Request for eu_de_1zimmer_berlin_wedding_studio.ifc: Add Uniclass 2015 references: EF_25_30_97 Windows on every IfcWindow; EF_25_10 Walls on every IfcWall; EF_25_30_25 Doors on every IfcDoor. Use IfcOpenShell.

First a look at what the model holds.

```python
import ifcopenshell

model = ifcopenshell.open("eu_de_1zimmer_berlin_wedding_studio.ifc")
print(model.schema)
print("classifications:", [c.Name for c in model.by_type("IfcClassification")])
for ifc_class in ("IfcDoor", "IfcRoof", "IfcStair", "IfcWall", "IfcWindow"):
    print(ifc_class, len(model.by_type(ifc_class)))
```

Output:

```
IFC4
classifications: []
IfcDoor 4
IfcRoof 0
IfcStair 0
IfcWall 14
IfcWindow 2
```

```python
import ifcopenshell
import ifcopenshell.api.classification

model = ifcopenshell.open("eu_de_1zimmer_berlin_wedding_studio.ifc")

system = ifcopenshell.api.classification.add_classification(model, classification="Uniclass 2015")

codes = {
    "IfcWindow": ("EF_25_30_97", "Windows"),
    "IfcWall": ("EF_25_10", "Walls"),
    "IfcDoor": ("EF_25_30_25", "Doors"),
}
for ifc_class, (code, name) in codes.items():
    products = model.by_type(ifc_class)
    ifcopenshell.api.classification.add_reference(
        model, products=products, classification=system, identification=code, name=name
    )
    print(code, len(products))

model.write("eu_de_1zimmer_berlin_wedding_studio-out.ifc")
```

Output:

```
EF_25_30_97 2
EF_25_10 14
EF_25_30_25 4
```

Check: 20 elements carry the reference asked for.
